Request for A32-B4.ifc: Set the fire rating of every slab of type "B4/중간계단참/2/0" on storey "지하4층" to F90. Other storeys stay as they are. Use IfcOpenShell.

First a look at what the model holds.

```python
import ifcopenshell
import ifcopenshell.util.element

model = ifcopenshell.open("A32-B4.ifc")
print(model.schema)
storey = next(s for s in model.by_type("IfcBuildingStorey") if s.Name == "지하4층")
slabs = [e for e in ifcopenshell.util.element.get_decomposition(storey) if e.is_a("IfcSlab")]
seen = {}
for e in slabs:
    element_type = ifcopenshell.util.element.get_type(e)
    key = (element_type.Name if element_type != e and element_type else None, ifcopenshell.util.element.get_pset(e, "Pset_SlabCommon", "FireRating"))
    seen[key] = seen.get(key, 0) + 1
for (name, value), count in sorted(seen.items(), key=str):
    print(count, "x", name, "|", value)
```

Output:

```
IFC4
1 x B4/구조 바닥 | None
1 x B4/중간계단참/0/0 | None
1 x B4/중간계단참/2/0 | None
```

```python
import ifcopenshell
import ifcopenshell.api.pset
import ifcopenshell.util.element

model = ifcopenshell.open("A32-B4.ifc")

storey = next(s for s in model.by_type("IfcBuildingStorey") if s.Name == "지하4층")
slabs = [e for e in ifcopenshell.util.element.get_decomposition(storey) if e.is_a("IfcSlab")]

count = 0
for e in slabs:
    element_type = ifcopenshell.util.element.get_type(e)
    if element_type in (None, e) or element_type.Name != "B4/중간계단참/2/0":
        continue
    # add_pset returns the element's existing set when there is one.
    pset = ifcopenshell.api.pset.add_pset(model, product=e, name="Pset_SlabCommon")
    ifcopenshell.api.pset.edit_pset(model, pset=pset, properties={"FireRating": "F90"})
    count += 1

print(count, "slabs updated")

model.write("A32-B4_rev.ifc")
```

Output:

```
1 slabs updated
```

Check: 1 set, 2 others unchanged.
